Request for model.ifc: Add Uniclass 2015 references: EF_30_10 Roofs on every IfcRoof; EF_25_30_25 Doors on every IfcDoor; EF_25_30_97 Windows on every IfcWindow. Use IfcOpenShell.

First a look at what the model holds.

```python
import ifcopenshell

model = ifcopenshell.open("model.ifc")
print(model.schema)
print("classifications:", [c.Name for c in model.by_type("IfcClassification")])
for ifc_class in ("IfcDoor", "IfcRoof", "IfcStair", "IfcWall", "IfcWindow"):
    print(ifc_class, len(model.by_type(ifc_class)))
```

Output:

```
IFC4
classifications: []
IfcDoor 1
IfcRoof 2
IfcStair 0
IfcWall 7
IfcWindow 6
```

```python
import ifcopenshell
import ifcopenshell.api.classification

model = ifcopenshell.open("model.ifc")

system = ifcopenshell.api.classification.add_classification(model, classification="Uniclass 2015")

codes = {
    "IfcRoof": ("EF_30_10", "Roofs"),
    "IfcDoor": ("EF_25_30_25", "Doors"),
    "IfcWindow": ("EF_25_30_97", "Windows"),
}
for ifc_class, (code, name) in codes.items():
    products = model.by_type(ifc_class)
    ifcopenshell.api.classification.add_reference(
        model, products=products, classification=system, identification=code, name=name
    )
    print(code, len(products))

model.write("model_edited.ifc")
```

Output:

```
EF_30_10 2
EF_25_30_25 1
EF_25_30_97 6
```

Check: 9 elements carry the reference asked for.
